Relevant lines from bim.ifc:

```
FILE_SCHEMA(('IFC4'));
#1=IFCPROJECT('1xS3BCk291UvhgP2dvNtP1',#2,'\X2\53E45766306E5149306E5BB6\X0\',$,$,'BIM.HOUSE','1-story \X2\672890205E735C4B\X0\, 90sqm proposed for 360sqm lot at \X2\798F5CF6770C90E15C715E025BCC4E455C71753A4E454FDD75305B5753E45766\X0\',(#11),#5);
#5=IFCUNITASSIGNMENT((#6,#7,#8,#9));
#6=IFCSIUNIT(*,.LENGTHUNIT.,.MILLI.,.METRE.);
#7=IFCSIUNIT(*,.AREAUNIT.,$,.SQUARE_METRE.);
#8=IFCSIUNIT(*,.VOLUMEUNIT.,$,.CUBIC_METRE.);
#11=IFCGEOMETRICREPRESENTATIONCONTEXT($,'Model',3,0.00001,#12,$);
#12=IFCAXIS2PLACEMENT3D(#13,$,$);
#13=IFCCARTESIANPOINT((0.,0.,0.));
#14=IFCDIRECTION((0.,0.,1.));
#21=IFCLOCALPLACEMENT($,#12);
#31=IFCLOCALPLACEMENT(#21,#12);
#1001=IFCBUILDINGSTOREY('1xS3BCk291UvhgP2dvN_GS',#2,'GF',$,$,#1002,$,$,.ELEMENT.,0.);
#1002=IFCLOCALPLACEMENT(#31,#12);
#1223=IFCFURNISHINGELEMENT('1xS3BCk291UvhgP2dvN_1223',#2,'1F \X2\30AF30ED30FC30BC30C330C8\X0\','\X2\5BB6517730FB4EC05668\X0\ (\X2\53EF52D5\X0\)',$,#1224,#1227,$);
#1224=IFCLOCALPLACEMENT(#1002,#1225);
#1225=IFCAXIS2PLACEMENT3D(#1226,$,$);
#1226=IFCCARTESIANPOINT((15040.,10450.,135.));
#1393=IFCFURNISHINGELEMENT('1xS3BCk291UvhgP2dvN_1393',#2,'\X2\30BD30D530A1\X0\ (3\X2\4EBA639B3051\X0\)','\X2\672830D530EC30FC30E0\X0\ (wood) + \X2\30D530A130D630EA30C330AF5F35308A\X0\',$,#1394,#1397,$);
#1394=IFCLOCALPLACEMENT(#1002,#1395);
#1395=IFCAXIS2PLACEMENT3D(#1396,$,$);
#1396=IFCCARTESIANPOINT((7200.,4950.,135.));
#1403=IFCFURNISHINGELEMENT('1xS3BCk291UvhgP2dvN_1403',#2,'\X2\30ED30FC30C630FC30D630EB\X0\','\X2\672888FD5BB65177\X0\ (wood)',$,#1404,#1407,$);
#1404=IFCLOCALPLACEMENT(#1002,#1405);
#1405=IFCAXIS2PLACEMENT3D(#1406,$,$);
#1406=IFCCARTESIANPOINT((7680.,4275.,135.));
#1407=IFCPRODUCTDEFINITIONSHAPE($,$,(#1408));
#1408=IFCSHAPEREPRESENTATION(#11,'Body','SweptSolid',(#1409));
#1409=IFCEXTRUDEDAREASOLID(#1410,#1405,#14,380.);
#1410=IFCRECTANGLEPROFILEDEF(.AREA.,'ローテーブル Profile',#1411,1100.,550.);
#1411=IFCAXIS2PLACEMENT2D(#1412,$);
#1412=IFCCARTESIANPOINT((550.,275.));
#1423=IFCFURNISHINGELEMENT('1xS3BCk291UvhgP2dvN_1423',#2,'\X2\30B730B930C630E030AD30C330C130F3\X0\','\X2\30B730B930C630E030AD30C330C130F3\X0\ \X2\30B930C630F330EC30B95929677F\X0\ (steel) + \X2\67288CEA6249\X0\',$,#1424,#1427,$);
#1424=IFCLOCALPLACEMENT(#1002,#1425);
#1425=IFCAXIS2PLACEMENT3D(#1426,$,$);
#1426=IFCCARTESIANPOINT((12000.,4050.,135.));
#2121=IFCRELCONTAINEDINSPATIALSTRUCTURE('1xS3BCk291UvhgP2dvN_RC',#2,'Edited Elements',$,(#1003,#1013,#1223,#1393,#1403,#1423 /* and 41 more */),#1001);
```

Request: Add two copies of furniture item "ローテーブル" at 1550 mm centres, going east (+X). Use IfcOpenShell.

```python
import numpy as np
import ifcopenshell
import ifcopenshell.api.geometry
import ifcopenshell.api.root
import ifcopenshell.util.element
import ifcopenshell.util.placement
import ifcopenshell.util.unit

model = ifcopenshell.open("bim.ifc")
unit_scale = ifcopenshell.util.unit.calculate_unit_scale(model)


def reuse_history(source, copy):
    """copy_class also copies each property set's owner history, people and application; keep the originals."""
    for rel in copy.IsDefinedBy:
        if rel.is_a("IfcRelDefinesByProperties") and (history := rel.RelatingPropertyDefinition.OwnerHistory):
            rel.RelatingPropertyDefinition.OwnerHistory = source.OwnerHistory
            ifcopenshell.util.element.remove_deep2(model, history)


source = model.by_guid("1xS3BCk291UvhgP2dvN_1403")
base = ifcopenshell.util.placement.get_local_placement(source.ObjectPlacement)
step = np.array([1.0, 0.0, 0.0]) * 1.55 / unit_scale

for i in range(1, 3):
    copy = ifcopenshell.api.root.copy_class(model, product=source)
    copy.Representation = ifcopenshell.util.element.copy_deep(
        model, source.Representation, exclude=["IfcGeometricRepresentationContext", "IfcRepresentationMap"]
    )
    reuse_history(source, copy)
    matrix = base.copy()
    matrix[:3, 3] += i * step
    print("added at", matrix[:3, 3].round(3) + 0.0)
    ifcopenshell.api.geometry.edit_object_placement(model, product=copy, matrix=matrix, is_si=False)

model.write("bim_v2.ifc")
```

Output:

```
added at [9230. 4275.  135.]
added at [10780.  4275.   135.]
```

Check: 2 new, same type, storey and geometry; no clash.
